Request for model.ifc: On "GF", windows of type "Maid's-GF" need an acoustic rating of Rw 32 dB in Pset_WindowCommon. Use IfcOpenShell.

First a look at what the model holds.

```python
import ifcopenshell
import ifcopenshell.util.element

model = ifcopenshell.open("model.ifc")
print(model.schema)
storey = next(s for s in model.by_type("IfcBuildingStorey") if s.Name == "GF")
windows = [e for e in ifcopenshell.util.element.get_decomposition(storey) if e.is_a("IfcWindow")]
seen = {}
for e in windows:
    element_type = ifcopenshell.util.element.get_type(e)
    key = (element_type.Name if element_type != e and element_type else None, ifcopenshell.util.element.get_pset(e, "Pset_WindowCommon", "AcousticRating"))
    seen[key] = seen.get(key, 0) + 1
for (name, value), count in sorted(seen.items(), key=str):
    print(count, "x", name, "|", value)
```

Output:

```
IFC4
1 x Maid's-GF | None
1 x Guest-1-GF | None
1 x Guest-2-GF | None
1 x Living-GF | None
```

```python
import ifcopenshell
import ifcopenshell.api.pset
import ifcopenshell.util.element

model = ifcopenshell.open("model.ifc")

storey = next(s for s in model.by_type("IfcBuildingStorey") if s.Name == "GF")
windows = [e for e in ifcopenshell.util.element.get_decomposition(storey) if e.is_a("IfcWindow")]

count = 0
for e in windows:
    element_type = ifcopenshell.util.element.get_type(e)
    if element_type in (None, e) or element_type.Name != "Maid's-GF":
        continue
    # add_pset returns the element's existing set when there is one.
    pset = ifcopenshell.api.pset.add_pset(model, product=e, name="Pset_WindowCommon")
    ifcopenshell.api.pset.edit_pset(model, pset=pset, properties={"AcousticRating": "Rw 32 dB"})
    count += 1

print(count, "windows updated")

model.write("model-out.ifc")
```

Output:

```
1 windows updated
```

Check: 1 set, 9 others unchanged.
